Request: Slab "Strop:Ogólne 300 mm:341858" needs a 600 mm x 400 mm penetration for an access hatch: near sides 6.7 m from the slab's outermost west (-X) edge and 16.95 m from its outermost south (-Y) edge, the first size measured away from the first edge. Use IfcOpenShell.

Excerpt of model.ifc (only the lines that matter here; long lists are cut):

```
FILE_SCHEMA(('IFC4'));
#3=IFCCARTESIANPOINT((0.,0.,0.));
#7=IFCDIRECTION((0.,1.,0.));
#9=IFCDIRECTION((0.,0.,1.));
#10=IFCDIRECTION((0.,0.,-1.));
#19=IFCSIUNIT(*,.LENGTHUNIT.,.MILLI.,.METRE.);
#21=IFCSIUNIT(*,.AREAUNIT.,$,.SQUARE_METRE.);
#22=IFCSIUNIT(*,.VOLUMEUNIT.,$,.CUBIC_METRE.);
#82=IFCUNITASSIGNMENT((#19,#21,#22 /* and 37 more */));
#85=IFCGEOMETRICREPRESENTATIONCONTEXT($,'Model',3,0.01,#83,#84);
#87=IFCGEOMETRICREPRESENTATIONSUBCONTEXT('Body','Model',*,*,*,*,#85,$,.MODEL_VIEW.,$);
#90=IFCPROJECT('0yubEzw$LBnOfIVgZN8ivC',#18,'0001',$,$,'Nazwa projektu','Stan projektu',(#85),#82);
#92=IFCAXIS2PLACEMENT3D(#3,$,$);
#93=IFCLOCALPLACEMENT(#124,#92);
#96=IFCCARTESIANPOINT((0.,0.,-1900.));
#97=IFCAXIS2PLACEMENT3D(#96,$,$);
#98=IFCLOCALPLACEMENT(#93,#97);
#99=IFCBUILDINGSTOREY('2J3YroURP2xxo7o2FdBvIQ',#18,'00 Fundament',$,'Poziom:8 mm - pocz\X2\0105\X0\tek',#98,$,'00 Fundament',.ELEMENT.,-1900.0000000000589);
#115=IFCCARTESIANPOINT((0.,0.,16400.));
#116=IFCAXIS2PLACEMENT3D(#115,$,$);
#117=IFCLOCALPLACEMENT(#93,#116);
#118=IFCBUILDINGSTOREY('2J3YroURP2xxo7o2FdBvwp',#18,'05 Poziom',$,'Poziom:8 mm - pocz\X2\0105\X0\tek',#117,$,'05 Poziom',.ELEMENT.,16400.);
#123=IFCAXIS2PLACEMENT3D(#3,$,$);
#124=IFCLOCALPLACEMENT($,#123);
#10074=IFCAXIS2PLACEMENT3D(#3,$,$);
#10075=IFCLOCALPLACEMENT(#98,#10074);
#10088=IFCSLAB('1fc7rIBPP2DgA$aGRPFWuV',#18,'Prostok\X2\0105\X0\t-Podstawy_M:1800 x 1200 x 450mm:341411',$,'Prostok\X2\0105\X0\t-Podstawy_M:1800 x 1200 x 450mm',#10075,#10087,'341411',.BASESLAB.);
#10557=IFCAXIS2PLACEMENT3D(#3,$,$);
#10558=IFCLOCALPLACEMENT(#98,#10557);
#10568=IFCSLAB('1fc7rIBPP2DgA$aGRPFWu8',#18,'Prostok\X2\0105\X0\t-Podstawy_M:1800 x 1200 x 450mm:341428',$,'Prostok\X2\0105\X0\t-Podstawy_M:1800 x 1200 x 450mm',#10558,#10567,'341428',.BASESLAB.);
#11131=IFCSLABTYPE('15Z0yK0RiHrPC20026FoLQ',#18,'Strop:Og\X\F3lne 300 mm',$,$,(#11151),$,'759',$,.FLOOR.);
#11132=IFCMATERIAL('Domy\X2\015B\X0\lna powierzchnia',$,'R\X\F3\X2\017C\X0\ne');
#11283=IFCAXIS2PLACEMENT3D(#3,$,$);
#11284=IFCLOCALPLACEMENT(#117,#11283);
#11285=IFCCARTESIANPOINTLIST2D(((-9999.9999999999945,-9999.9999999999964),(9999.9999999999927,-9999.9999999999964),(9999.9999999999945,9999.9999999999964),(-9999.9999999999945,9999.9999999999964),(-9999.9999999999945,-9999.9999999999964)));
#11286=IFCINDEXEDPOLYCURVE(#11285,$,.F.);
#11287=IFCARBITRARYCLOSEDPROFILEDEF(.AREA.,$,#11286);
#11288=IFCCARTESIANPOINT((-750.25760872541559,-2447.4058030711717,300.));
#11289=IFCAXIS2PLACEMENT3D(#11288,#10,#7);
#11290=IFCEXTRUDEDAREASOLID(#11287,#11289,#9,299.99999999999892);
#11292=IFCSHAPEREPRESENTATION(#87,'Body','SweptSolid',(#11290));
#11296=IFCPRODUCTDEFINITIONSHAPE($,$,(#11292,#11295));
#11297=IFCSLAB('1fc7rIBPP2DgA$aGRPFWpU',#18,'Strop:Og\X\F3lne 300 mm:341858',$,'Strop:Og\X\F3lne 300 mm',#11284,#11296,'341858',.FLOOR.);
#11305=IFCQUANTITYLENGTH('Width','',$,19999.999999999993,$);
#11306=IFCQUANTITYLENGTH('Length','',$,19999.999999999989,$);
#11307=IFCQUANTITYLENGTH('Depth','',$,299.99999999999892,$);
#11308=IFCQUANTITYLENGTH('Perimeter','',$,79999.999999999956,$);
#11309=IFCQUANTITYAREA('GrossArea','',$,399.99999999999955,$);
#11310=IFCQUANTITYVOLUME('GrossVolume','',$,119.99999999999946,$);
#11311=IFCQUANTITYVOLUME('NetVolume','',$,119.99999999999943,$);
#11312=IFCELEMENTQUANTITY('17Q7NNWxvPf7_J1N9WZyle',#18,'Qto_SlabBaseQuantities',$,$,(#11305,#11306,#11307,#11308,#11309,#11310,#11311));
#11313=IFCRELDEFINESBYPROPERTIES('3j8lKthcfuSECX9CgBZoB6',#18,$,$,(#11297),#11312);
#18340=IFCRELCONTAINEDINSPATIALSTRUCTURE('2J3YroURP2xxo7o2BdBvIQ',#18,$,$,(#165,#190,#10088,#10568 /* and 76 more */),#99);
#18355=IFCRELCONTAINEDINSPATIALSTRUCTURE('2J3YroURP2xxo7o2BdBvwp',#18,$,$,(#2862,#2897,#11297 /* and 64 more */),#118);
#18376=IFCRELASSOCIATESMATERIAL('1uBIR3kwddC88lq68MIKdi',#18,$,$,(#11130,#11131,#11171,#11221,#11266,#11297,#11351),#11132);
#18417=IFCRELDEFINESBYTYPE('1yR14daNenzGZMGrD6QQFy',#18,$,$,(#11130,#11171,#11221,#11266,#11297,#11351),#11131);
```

```python
import numpy as np
import ifcopenshell
import ifcopenshell.api.feature
import ifcopenshell.api.geometry
import ifcopenshell.api.pset
import ifcopenshell.api.root
import ifcopenshell.geom
import ifcopenshell.util.element
import ifcopenshell.util.placement
import ifcopenshell.util.representation
import ifcopenshell.util.shape
import ifcopenshell.util.unit

model = ifcopenshell.open("model.ifc")
unit_scale = ifcopenshell.util.unit.calculate_unit_scale(model)
volume_scale = ifcopenshell.util.unit.calculate_unit_scale(model, "VOLUMEUNIT")
settings = ifcopenshell.geom.settings()


def volume(element):
    """Net volume in cubic metres, openings subtracted."""
    shape = ifcopenshell.geom.create_shape(settings, element)
    return ifcopenshell.util.shape.get_volume(shape.geometry)


slab = model.by_guid("1fc7rIBPP2DgA$aGRPFWpU")
before = volume(slab)

# Extent in the slab's own axes, in metres. The edges named are its -X and -Y sides.
slab_shape = ifcopenshell.geom.create_shape(settings, slab)
vertices = ifcopenshell.util.shape.get_vertices(slab_shape.geometry)
x_min, y_min, bottom = vertices.min(axis=0)
top = vertices[:, 2].max()

opening = ifcopenshell.api.root.create_entity(model, ifc_class="IfcOpeningElement", name="Access hatch opening", predefined_type="OPENING")
context = ifcopenshell.util.representation.get_context(model, "Model", "Body", "MODEL_VIEW")
width, depth = 0.6, 0.4
outline = [(0.0, 0.0), (width, 0.0), (width, depth), (0.0, depth), (0.0, 0.0)]
# Overshoot both faces by 50 mm so the cut is clean.
shape = ifcopenshell.api.geometry.add_slab_representation(
    model, context=context, depth=top - bottom + 0.1, polyline=outline
)
ifcopenshell.api.geometry.assign_representation(model, product=opening, representation=shape)

matrix = ifcopenshell.util.placement.get_local_placement(slab.ObjectPlacement)
matrix[:, 3] = matrix @ np.append(np.array([x_min + 6.7, y_min + 16.95, bottom - 0.05]) / unit_scale, 1.0)
ifcopenshell.api.geometry.edit_object_placement(model, product=opening, matrix=matrix, is_si=False)
ifcopenshell.api.feature.add_feature(model, feature=opening, element=slab)

after = volume(slab)

# Update the slab's stored quantities.
qto = model.by_id(ifcopenshell.util.element.get_pset(slab, "Qto_SlabBaseQuantities", should_inherit=False)["id"])
ifcopenshell.api.pset.edit_qto(model, qto=qto, properties={"NetVolume": after / volume_scale})

print(f"slab volume {before:.3f} -> {after:.3f} m3")

model.write("model_edited.ifc")
```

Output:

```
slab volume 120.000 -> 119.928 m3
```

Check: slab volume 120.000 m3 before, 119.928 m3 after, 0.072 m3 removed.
